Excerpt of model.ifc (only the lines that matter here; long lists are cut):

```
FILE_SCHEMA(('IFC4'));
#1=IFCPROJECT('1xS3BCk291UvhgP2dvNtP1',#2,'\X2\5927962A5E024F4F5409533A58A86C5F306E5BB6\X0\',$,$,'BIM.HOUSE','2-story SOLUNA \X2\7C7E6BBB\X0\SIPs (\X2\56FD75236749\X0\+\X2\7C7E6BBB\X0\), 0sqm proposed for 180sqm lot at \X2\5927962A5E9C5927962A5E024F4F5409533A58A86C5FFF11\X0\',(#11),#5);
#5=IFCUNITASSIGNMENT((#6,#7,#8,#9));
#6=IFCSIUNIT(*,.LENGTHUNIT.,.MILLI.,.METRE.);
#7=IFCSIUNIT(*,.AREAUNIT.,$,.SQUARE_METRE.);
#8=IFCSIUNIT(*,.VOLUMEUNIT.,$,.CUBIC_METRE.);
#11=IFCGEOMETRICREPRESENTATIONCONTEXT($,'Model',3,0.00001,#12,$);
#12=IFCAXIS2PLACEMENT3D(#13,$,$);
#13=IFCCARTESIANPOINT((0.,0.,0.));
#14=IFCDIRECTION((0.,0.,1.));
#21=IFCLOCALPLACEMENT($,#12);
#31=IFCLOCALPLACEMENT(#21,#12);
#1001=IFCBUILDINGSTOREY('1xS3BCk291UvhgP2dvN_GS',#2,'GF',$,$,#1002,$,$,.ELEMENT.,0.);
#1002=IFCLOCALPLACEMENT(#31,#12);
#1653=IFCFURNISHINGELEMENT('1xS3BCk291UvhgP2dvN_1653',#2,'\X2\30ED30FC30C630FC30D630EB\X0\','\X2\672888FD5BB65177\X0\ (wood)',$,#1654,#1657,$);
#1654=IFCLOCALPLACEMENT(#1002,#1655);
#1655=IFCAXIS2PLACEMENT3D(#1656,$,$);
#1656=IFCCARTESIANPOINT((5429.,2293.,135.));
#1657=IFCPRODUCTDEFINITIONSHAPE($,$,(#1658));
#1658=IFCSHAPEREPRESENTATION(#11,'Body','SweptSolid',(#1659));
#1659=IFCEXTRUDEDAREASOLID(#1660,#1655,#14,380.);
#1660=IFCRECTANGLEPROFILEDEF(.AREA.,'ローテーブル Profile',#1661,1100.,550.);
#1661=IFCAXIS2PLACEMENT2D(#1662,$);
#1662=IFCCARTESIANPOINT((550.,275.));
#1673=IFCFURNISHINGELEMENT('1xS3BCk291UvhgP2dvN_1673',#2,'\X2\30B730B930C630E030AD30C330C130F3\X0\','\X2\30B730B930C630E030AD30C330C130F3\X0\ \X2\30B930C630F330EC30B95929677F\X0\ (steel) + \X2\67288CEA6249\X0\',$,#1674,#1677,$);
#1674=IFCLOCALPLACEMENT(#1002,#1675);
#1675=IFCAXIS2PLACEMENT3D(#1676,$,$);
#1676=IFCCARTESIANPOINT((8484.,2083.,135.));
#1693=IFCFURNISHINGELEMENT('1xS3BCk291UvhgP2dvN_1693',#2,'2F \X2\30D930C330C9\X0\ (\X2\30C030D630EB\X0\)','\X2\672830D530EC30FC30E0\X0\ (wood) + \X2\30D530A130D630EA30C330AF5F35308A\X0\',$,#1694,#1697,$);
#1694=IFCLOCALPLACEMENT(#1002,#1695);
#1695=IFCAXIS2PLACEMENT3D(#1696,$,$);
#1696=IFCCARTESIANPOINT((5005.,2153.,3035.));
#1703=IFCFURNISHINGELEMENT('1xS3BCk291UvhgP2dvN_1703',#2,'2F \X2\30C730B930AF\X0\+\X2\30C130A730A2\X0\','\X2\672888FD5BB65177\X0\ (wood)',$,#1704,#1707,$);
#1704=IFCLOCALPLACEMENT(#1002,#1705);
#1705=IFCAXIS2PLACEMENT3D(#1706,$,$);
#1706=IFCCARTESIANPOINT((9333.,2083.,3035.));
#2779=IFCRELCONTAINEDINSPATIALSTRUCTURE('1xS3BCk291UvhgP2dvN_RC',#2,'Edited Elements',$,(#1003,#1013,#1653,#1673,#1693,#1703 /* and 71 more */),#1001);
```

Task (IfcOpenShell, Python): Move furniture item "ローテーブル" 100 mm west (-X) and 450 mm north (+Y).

```python
import ifcopenshell
import ifcopenshell.api.geometry
import ifcopenshell.util.placement

model = ifcopenshell.open("model.ifc")

item = model.by_id(1653)
matrix = ifcopenshell.util.placement.get_local_placement(item.ObjectPlacement)
matrix[0, 3] -= 100.0
matrix[1, 3] += 450.0
ifcopenshell.api.geometry.edit_object_placement(model, product=item, matrix=matrix, is_si=False)

print(ifcopenshell.util.placement.get_local_placement(item.ObjectPlacement).round(3) + 0.0)

model.write("model_rev.ifc")
```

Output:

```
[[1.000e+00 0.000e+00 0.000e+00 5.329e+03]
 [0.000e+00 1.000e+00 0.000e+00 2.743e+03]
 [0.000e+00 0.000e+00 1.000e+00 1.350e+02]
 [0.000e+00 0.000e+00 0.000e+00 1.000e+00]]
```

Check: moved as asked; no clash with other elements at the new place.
